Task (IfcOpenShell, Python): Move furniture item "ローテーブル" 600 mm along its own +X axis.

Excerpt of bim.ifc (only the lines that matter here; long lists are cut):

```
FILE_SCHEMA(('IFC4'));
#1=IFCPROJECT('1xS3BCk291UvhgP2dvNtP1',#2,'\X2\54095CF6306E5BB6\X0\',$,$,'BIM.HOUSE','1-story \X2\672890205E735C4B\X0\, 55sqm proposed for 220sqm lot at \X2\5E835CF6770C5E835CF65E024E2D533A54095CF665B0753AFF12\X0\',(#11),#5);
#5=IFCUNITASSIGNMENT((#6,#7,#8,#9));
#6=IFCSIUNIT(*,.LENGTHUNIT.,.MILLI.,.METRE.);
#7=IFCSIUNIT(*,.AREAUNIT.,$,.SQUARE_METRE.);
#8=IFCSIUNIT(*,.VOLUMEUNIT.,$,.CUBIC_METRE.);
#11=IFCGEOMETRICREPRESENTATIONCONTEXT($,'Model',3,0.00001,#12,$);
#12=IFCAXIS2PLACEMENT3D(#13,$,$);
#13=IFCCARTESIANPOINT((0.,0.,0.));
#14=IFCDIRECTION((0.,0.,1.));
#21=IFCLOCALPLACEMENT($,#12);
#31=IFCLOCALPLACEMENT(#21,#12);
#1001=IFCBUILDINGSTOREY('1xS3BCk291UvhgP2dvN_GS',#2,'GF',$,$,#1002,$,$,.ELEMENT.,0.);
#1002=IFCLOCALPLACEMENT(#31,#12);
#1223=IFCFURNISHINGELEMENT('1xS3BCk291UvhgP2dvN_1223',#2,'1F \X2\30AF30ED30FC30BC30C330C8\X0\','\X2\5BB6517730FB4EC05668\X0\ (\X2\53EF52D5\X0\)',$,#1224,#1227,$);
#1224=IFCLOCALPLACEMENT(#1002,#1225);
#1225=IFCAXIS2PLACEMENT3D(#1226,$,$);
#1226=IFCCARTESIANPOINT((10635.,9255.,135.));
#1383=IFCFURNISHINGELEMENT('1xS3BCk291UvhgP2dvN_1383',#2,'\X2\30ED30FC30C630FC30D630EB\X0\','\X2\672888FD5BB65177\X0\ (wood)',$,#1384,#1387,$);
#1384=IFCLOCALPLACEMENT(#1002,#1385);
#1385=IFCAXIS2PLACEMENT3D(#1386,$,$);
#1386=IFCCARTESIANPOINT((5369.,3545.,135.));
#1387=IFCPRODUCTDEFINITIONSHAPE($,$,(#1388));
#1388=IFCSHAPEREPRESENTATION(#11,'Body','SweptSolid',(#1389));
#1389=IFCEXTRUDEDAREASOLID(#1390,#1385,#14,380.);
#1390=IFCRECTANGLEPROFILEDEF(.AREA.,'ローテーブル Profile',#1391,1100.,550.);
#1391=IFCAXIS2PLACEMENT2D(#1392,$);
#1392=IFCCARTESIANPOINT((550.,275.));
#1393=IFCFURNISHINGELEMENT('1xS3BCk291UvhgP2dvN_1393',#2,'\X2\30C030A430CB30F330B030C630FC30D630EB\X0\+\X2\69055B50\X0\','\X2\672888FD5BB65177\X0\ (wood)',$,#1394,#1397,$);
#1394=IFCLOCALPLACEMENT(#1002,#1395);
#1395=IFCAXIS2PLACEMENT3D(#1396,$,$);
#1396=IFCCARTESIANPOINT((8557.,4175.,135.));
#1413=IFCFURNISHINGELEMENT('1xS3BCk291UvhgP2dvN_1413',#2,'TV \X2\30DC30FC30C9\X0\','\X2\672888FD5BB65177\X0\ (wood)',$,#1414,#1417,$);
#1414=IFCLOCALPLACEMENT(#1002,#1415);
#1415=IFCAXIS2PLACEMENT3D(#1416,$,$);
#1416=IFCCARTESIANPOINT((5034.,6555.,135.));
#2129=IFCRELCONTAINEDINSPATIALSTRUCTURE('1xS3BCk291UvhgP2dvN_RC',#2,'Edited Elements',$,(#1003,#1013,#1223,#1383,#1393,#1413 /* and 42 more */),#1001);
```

```python
import ifcopenshell
import ifcopenshell.api.geometry
import ifcopenshell.util.placement
import ifcopenshell.util.unit

model = ifcopenshell.open("bim.ifc")
unit_scale = ifcopenshell.util.unit.calculate_unit_scale(model)

item = model.by_id(1383)
matrix = ifcopenshell.util.placement.get_local_placement(item.ObjectPlacement)
matrix[:3, 3] += matrix[:3, 0] * 0.6 / unit_scale
ifcopenshell.api.geometry.edit_object_placement(model, product=item, matrix=matrix, is_si=False)

print(ifcopenshell.util.placement.get_local_placement(item.ObjectPlacement).round(3) + 0.0)

model.write("bim_rev.ifc")
```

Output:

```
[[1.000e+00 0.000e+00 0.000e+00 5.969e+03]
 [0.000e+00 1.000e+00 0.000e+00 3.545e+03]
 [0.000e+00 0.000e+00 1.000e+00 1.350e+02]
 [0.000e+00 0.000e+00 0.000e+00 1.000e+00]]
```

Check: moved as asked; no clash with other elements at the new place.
